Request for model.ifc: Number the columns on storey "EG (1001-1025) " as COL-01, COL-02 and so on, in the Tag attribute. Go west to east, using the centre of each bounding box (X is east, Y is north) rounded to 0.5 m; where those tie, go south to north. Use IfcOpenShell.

First a look at what the model holds.

```python
import ifcopenshell
import ifcopenshell.util.element
import ifcopenshell.util.placement

model = ifcopenshell.open("model.ifc")
print(model.schema)
storey = next(s for s in model.by_type("IfcBuildingStorey") if s.Name == "EG (1001-1025) ")
columns = [e for e in ifcopenshell.util.element.get_decomposition(storey) if e.is_a("IfcColumn")]
for e in sorted(columns, key=lambda e: e.id()):
    origin = ifcopenshell.util.placement.get_local_placement(e.ObjectPlacement)[:3, 3]
    print(e.id(), e.Tag, e.Name, origin.round(2) + 0.0, sep=" | ")
```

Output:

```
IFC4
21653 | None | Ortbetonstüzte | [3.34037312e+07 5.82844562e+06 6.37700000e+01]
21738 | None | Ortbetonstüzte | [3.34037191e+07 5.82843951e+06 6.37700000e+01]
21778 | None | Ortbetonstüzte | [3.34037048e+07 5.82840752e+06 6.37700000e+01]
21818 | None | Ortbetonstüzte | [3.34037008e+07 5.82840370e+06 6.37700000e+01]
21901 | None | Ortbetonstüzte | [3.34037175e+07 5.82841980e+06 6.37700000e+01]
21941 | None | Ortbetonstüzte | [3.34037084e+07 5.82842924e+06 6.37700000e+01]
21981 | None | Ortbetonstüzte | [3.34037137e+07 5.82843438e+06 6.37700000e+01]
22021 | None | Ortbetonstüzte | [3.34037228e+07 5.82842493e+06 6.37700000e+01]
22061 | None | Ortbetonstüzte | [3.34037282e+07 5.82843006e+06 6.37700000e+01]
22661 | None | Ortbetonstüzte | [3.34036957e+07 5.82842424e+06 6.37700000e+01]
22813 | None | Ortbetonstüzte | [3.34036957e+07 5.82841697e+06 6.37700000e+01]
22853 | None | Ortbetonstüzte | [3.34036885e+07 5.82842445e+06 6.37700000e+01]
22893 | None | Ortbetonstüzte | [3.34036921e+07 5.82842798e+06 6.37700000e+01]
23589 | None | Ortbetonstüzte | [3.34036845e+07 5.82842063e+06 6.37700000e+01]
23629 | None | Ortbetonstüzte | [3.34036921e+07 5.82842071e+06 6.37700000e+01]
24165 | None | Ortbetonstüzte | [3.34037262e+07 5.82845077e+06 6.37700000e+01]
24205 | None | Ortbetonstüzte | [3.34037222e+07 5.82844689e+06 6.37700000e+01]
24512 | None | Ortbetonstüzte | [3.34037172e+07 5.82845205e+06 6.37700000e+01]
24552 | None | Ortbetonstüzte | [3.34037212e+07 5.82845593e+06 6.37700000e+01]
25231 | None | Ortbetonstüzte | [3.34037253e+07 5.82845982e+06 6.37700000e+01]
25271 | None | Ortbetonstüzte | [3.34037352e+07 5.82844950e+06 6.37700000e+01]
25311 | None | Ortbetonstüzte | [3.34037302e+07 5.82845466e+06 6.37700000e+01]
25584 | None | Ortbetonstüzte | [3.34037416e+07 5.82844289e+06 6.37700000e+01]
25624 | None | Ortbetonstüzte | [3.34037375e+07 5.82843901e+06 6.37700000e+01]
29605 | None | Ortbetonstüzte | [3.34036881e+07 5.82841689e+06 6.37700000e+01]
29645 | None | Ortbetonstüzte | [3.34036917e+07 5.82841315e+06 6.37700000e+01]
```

```python
import ifcopenshell
import ifcopenshell.geom
import ifcopenshell.util.element
import ifcopenshell.util.shape

model = ifcopenshell.open("model.ifc")
settings = ifcopenshell.geom.settings()
settings.set("use-world-coords", True)


def centre(element):
    shape = ifcopenshell.geom.create_shape(settings, element)
    return ifcopenshell.util.shape.get_bbox_centroid(shape.geometry)


storey = next(s for s in model.by_type("IfcBuildingStorey") if s.Name == "EG (1001-1025) ")
columns = [e for e in ifcopenshell.util.element.get_decomposition(storey) if e.is_a("IfcColumn")]

# Insertion points can sit at a corner or the storey origin, so sort by the geometry (in metres).
centres = {e: centre(e) for e in columns}
columns.sort(key=lambda e: (round(centres[e][0] / 0.5), centres[e][1]))

for i, e in enumerate(columns, start=1):
    number = f"COL-{i:02d}"
    e.Tag = number
    print(e.id(), number)

model.write("model_rev.ifc")
```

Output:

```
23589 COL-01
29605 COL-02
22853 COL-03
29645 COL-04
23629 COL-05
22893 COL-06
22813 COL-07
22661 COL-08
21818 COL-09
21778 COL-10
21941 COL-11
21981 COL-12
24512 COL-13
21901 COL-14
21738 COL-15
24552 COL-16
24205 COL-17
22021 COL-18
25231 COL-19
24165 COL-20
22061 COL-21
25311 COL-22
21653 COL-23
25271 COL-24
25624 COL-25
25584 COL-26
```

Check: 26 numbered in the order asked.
